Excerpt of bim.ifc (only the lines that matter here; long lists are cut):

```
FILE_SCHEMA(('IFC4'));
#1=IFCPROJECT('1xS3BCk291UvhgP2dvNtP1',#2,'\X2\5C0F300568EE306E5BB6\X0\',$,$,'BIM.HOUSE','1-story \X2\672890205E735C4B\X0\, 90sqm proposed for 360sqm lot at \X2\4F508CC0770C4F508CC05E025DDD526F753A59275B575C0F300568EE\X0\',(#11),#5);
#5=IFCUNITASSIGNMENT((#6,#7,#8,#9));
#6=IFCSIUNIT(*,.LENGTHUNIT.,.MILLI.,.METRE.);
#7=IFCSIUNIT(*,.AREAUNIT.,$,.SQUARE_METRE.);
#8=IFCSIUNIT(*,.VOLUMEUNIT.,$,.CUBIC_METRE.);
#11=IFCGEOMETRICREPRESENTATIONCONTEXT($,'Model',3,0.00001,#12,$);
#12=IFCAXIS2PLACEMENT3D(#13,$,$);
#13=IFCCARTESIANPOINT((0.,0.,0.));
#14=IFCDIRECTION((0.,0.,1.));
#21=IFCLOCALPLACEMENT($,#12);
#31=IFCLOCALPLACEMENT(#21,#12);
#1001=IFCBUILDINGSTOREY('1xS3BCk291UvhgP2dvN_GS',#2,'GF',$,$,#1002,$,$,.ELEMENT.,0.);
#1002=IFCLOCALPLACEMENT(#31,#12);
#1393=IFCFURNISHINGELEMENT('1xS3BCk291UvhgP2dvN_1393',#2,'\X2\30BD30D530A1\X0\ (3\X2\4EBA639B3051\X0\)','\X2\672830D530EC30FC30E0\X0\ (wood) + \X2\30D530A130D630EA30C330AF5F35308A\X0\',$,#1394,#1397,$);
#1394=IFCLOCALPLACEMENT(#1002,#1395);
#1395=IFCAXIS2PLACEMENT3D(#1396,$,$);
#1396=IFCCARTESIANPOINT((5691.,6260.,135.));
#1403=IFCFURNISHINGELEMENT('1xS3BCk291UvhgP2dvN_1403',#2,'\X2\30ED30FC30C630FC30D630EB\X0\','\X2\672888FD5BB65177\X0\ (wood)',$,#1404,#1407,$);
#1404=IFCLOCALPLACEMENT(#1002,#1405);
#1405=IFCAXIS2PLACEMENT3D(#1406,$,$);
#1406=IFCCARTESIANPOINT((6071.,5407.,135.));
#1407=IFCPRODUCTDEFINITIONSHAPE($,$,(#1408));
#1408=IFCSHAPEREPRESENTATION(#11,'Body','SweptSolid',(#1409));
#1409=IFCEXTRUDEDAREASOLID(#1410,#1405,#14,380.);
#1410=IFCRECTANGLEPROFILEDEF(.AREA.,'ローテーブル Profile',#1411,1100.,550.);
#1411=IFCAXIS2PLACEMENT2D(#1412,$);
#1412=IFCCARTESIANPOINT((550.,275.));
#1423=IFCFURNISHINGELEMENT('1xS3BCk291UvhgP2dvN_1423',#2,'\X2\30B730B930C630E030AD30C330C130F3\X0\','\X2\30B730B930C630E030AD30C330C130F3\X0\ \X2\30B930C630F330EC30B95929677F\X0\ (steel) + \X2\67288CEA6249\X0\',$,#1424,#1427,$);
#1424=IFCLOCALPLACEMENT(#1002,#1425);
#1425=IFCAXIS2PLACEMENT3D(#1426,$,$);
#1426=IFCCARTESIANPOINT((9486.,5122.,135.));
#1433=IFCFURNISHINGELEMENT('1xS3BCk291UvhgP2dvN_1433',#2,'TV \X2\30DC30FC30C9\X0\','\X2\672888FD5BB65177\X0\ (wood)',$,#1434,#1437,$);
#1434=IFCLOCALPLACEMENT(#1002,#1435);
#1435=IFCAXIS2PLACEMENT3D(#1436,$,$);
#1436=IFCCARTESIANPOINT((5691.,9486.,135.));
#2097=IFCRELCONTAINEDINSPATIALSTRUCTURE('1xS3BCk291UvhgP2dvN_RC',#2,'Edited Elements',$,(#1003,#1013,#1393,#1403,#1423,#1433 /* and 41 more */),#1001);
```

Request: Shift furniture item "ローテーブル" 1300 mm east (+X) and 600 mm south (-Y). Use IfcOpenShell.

```python
import ifcopenshell
import ifcopenshell.api.geometry
import ifcopenshell.util.placement
import ifcopenshell.util.unit

model = ifcopenshell.open("bim.ifc")
unit_scale = ifcopenshell.util.unit.calculate_unit_scale(model)

item = model.by_guid("1xS3BCk291UvhgP2dvN_1403")
matrix = ifcopenshell.util.placement.get_local_placement(item.ObjectPlacement)
matrix[0, 3] += 1.3 / unit_scale
matrix[1, 3] -= 0.6 / unit_scale
ifcopenshell.api.geometry.edit_object_placement(model, product=item, matrix=matrix, is_si=False)

print(ifcopenshell.util.placement.get_local_placement(item.ObjectPlacement).round(3) + 0.0)

model.write("bim-out.ifc")
```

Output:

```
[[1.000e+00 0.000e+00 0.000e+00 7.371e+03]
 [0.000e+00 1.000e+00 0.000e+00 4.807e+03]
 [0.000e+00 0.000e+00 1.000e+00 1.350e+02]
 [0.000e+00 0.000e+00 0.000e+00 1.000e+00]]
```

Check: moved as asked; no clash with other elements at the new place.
